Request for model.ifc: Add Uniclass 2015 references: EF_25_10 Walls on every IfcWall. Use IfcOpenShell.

First a look at what the model holds.

```python
import ifcopenshell

model = ifcopenshell.open("model.ifc")
print(model.schema)
print("classifications:", [c.Name for c in model.by_type("IfcClassification")])
for ifc_class in ("IfcDoor", "IfcRoof", "IfcStair", "IfcWall", "IfcWindow"):
    print(ifc_class, len(model.by_type(ifc_class)))
```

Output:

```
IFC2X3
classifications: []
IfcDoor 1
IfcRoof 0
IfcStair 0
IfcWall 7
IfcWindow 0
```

```python
import ifcopenshell
import ifcopenshell.api.classification

model = ifcopenshell.open("model.ifc")

# IFC2X3 requires Source and Edition and has no link from the project to the system.
system = model.create_entity("IfcClassification", Source="NBS", Edition="2015", Name="Uniclass 2015")

codes = {
    "IfcWall": ("EF_25_10", "Walls"),
}
for ifc_class, (code, name) in codes.items():
    products = model.by_type(ifc_class)
    ifcopenshell.api.classification.add_reference(
        model, products=products, classification=system, identification=code, name=name
    )
    print(code, len(products))

model.write("model-out.ifc")
```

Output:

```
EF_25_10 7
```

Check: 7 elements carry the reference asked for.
